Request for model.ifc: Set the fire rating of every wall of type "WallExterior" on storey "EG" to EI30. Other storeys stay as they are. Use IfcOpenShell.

First a look at what the model holds.

```python
import ifcopenshell
import ifcopenshell.util.element

model = ifcopenshell.open("model.ifc")
print(model.schema)
storey = next(s for s in model.by_type("IfcBuildingStorey") if s.Name == "EG")
walls = [e for e in ifcopenshell.util.element.get_decomposition(storey) if e.is_a("IfcWall")]
seen = {}
for e in walls:
    element_type = ifcopenshell.util.element.get_type(e)
    key = (element_type.Name if element_type != e and element_type else None, ifcopenshell.util.element.get_pset(e, "Pset_WallCommon", "FireRating"))
    seen[key] = seen.get(key, 0) + 1
for (name, value), count in sorted(seen.items(), key=str):
    print(count, "x", name, "|", value)
```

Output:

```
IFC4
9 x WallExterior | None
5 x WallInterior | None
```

```python
import ifcopenshell
import ifcopenshell.api.pset
import ifcopenshell.util.element

model = ifcopenshell.open("model.ifc")

storey = next(s for s in model.by_type("IfcBuildingStorey") if s.Name == "EG")
walls = [e for e in ifcopenshell.util.element.get_decomposition(storey) if e.is_a("IfcWall")]

count = 0
for e in walls:
    element_type = ifcopenshell.util.element.get_type(e)
    if element_type in (None, e) or element_type.Name != "WallExterior":
        continue
    # add_pset returns the element's existing set when there is one.
    pset = ifcopenshell.api.pset.add_pset(model, product=e, name="Pset_WallCommon")
    ifcopenshell.api.pset.edit_pset(model, pset=pset, properties={"FireRating": "EI30"})
    count += 1

print(count, "walls updated")

model.write("model-out.ifc")
```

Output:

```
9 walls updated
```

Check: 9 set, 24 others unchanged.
